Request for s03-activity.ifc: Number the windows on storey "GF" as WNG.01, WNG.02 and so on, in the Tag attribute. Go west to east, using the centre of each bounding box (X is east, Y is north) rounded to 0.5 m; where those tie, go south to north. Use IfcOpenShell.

First a look at what the model holds.

```python
import ifcopenshell
import ifcopenshell.util.element
import ifcopenshell.util.placement

model = ifcopenshell.open("s03-activity.ifc")
print(model.schema)
storey = next(s for s in model.by_type("IfcBuildingStorey") if s.Name == "GF")
windows = [e for e in ifcopenshell.util.element.get_decomposition(storey) if e.is_a("IfcWindow")]
for e in sorted(windows, key=lambda e: e.id()):
    origin = ifcopenshell.util.placement.get_local_placement(e.ObjectPlacement)[:3, 3]
    print(e.id(), e.Tag, e.Name, origin.round(2) + 0.0, sep=" | ")
```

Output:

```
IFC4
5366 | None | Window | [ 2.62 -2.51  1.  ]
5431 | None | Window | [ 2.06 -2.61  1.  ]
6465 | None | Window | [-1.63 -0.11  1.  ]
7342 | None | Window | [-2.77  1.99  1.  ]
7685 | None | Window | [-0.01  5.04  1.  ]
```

```python
import ifcopenshell
import ifcopenshell.geom
import ifcopenshell.util.element
import ifcopenshell.util.shape

model = ifcopenshell.open("s03-activity.ifc")
settings = ifcopenshell.geom.settings()
settings.set("use-world-coords", True)


def centre(element):
    shape = ifcopenshell.geom.create_shape(settings, element)
    return ifcopenshell.util.shape.get_bbox_centroid(shape.geometry)


storey = next(s for s in model.by_type("IfcBuildingStorey") if s.Name == "GF")
windows = [e for e in ifcopenshell.util.element.get_decomposition(storey) if e.is_a("IfcWindow")]

# Insertion points can sit at a corner or the storey origin, so sort by the geometry (in metres).
centres = {e: centre(e) for e in windows}
windows.sort(key=lambda e: (round(centres[e][0] / 0.5), centres[e][1]))

for i, e in enumerate(windows, start=1):
    number = f"WNG.{i:02d}"
    e.Tag = number
    print(e.id(), number)

model.write("s03-activity_edited.ifc")
```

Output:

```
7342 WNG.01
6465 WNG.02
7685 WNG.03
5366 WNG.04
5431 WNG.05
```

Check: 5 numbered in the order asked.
